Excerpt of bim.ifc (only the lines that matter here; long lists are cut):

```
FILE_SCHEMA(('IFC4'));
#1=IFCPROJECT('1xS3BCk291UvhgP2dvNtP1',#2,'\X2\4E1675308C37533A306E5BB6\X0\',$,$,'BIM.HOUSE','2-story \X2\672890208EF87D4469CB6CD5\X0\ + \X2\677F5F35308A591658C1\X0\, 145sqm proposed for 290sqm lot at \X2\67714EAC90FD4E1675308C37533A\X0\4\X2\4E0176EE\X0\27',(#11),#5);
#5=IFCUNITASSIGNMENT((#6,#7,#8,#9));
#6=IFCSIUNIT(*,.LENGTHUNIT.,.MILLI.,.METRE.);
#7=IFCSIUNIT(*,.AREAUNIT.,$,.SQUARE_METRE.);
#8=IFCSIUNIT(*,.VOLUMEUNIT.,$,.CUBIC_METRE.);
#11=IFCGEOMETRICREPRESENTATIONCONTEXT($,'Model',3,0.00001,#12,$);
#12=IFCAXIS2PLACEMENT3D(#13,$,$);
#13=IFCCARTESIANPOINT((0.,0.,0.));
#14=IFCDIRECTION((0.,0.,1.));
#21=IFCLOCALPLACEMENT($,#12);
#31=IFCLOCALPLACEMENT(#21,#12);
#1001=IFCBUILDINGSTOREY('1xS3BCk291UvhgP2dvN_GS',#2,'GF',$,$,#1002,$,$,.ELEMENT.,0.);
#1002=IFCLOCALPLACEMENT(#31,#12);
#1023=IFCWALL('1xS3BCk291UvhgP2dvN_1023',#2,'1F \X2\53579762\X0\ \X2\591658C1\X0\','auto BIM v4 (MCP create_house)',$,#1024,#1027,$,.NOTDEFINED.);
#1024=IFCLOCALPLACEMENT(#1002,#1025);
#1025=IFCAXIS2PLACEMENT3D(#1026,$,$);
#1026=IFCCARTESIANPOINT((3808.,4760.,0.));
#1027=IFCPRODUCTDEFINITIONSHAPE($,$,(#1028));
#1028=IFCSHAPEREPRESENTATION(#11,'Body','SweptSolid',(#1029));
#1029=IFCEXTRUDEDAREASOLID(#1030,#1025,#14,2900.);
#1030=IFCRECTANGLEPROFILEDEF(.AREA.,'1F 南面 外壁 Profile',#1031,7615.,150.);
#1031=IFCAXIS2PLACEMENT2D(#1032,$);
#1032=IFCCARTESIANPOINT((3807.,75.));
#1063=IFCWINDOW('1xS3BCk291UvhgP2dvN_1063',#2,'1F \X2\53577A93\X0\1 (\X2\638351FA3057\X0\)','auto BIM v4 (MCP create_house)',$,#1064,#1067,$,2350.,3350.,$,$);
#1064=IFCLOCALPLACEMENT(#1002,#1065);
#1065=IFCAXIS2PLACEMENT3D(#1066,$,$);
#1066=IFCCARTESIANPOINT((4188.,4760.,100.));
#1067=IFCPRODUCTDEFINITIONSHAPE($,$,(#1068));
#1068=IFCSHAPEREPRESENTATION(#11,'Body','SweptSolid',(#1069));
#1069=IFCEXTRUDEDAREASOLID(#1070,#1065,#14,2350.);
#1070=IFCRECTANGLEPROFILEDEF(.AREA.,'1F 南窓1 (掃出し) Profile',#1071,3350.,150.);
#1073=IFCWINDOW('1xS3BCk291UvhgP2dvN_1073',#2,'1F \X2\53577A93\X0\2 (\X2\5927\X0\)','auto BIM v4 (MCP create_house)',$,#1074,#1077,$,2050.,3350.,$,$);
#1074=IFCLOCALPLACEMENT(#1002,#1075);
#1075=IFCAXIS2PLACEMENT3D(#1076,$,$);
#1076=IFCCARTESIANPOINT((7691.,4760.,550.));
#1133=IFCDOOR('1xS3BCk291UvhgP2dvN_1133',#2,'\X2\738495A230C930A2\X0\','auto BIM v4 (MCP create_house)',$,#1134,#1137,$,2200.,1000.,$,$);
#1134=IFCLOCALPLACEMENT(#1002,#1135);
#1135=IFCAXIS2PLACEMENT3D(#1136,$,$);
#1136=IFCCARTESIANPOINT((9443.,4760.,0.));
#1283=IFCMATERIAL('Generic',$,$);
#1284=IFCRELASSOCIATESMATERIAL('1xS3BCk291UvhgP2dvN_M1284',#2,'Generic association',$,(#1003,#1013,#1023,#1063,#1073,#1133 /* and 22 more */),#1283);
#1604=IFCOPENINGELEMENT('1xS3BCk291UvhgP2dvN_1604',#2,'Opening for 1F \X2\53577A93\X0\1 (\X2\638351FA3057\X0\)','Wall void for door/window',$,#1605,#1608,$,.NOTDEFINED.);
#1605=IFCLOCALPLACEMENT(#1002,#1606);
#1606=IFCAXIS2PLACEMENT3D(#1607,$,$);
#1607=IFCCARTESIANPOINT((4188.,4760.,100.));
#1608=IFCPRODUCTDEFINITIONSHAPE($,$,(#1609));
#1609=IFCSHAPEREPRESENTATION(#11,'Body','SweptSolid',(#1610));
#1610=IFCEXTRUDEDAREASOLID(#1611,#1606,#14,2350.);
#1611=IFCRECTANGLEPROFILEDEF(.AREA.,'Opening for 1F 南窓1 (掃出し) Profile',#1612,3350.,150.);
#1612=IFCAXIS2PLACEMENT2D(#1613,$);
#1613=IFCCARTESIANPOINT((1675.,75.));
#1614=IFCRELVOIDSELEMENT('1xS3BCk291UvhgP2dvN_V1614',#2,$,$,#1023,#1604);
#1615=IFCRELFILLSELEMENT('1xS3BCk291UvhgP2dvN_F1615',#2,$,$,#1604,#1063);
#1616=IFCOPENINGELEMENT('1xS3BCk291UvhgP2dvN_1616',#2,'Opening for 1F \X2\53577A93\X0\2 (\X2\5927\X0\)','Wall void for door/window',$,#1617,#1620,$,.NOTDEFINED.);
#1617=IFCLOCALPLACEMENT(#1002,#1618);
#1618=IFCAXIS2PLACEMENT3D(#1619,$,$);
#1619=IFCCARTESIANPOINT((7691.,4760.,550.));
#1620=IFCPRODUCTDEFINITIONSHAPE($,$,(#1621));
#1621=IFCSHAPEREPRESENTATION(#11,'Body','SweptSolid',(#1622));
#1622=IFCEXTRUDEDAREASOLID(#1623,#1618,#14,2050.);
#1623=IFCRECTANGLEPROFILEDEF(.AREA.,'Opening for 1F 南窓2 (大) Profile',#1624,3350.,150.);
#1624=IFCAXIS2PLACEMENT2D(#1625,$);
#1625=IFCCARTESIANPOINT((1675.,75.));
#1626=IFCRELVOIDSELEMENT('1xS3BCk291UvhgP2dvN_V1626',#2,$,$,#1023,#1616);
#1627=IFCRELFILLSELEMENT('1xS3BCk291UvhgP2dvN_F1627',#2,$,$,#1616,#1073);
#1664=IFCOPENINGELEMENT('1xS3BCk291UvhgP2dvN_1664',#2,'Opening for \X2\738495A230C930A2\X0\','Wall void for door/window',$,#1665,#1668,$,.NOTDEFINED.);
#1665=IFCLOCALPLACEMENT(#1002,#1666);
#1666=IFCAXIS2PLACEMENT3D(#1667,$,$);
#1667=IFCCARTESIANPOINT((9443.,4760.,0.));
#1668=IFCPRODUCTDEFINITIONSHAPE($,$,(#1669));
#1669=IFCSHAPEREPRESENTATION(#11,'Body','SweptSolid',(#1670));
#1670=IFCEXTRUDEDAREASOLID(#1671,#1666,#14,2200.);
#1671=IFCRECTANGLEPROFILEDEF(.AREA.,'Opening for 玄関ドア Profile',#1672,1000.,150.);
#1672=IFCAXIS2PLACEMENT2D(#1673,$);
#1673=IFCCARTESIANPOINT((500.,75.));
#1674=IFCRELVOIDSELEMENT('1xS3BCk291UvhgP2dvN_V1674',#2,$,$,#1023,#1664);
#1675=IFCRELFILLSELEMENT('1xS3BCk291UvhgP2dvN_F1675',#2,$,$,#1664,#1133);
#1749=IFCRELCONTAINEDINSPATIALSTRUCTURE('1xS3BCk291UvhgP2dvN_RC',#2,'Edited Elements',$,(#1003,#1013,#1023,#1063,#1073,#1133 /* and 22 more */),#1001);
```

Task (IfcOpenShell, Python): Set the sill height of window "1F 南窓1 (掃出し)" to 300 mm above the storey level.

```python
import numpy as np
import ifcopenshell
import ifcopenshell.api.geometry
import ifcopenshell.geom
import ifcopenshell.util.element
import ifcopenshell.util.placement
import ifcopenshell.util.shape
import ifcopenshell.util.unit

model = ifcopenshell.open("bim.ifc")
unit_scale = ifcopenshell.util.unit.calculate_unit_scale(model)

window = model.by_id(1063)
opening = window.FillsVoids[0].RelatingOpeningElement
storey = ifcopenshell.util.element.get_container(window, ifc_class="IfcBuildingStorey")
level = ifcopenshell.util.placement.get_local_placement(storey.ObjectPlacement)[2, 3]

# The opening's origin need not be at the sill, so measure its lowest point.
shape = ifcopenshell.geom.create_shape(ifcopenshell.geom.settings(), opening)
bottom = ifcopenshell.util.shape.get_shape_bottom_elevation(shape, shape.geometry) / unit_scale
dz = level + 300.0 - bottom

shift = np.array([0.0, 0.0, dz])
# The window is not placed relative to its opening, so move both.
for product in (opening, window):
    matrix = ifcopenshell.util.placement.get_local_placement(product.ObjectPlacement)
    matrix[:3, 3] += shift
    ifcopenshell.api.geometry.edit_object_placement(model, product=product, matrix=matrix, is_si=False)

print(f"moved by {dz * unit_scale:+.3f} m")

model.write("bim_rev.ifc")
```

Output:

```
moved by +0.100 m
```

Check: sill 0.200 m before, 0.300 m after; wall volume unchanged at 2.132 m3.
